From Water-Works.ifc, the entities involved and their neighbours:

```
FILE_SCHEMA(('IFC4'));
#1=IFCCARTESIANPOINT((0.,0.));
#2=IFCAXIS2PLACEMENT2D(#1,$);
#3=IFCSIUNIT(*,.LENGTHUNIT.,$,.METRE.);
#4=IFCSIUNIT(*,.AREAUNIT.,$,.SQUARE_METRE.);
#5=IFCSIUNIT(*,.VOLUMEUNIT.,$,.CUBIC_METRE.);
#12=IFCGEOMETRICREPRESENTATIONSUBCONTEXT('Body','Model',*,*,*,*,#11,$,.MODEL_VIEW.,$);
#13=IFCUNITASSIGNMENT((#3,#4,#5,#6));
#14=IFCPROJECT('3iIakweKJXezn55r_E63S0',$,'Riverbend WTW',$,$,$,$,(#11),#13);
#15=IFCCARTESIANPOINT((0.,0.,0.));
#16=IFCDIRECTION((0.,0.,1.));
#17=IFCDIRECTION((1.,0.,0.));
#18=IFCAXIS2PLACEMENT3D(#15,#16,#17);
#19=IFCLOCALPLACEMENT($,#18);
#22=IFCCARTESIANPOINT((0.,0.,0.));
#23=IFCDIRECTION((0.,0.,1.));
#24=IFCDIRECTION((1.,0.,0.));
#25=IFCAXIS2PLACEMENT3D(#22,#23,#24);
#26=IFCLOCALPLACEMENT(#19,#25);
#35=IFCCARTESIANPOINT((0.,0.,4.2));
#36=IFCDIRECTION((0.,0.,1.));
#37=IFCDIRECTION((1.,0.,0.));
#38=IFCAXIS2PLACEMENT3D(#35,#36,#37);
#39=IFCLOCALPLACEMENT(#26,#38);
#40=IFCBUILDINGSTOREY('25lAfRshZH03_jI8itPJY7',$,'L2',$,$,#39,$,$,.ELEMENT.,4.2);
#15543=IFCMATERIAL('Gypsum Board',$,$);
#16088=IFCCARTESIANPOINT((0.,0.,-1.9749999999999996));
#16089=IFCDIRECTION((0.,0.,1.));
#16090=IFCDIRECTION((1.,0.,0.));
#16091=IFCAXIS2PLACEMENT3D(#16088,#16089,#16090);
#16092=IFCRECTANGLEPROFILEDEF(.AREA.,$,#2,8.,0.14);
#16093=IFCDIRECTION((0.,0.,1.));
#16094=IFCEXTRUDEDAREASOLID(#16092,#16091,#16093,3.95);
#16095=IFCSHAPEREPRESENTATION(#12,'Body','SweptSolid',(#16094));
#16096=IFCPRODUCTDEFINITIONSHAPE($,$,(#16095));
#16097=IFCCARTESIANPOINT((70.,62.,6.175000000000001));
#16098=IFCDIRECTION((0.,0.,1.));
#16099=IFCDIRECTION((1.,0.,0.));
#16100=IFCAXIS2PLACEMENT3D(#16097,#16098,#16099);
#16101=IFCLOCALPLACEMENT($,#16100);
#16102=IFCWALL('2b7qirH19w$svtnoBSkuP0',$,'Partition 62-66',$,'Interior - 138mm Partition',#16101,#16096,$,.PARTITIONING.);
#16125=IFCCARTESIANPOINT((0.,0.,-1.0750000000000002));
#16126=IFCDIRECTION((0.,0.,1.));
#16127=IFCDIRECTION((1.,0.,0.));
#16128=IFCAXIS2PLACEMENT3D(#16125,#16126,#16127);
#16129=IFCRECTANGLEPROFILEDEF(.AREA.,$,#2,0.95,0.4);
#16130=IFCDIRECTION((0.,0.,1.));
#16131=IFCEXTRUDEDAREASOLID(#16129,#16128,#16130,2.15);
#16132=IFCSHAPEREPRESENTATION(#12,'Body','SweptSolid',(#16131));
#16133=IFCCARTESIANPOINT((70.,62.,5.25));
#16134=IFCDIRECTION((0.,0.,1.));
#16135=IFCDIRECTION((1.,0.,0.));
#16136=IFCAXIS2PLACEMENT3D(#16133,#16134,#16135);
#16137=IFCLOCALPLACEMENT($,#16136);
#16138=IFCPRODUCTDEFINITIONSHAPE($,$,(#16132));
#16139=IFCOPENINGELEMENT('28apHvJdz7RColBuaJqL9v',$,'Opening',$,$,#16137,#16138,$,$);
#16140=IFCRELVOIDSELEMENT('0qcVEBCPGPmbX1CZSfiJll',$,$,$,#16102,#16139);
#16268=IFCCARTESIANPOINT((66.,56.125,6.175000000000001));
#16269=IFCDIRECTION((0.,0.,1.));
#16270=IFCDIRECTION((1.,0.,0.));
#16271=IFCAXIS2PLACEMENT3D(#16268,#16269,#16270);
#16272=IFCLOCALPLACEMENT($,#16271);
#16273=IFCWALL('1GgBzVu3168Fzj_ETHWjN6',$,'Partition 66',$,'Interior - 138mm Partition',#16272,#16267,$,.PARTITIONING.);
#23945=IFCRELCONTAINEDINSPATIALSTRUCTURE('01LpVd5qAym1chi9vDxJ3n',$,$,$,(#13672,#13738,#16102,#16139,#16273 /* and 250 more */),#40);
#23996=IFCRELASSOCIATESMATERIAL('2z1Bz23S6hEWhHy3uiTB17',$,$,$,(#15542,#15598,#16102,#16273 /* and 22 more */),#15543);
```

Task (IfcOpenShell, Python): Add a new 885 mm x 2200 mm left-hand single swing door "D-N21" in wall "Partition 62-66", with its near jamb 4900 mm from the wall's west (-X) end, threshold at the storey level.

```python
import numpy as np
import ifcopenshell
import ifcopenshell.api.feature
import ifcopenshell.api.geometry
import ifcopenshell.api.root
import ifcopenshell.api.spatial
import ifcopenshell.geom
import ifcopenshell.util.element
import ifcopenshell.util.placement
import ifcopenshell.util.representation
import ifcopenshell.util.shape
import ifcopenshell.util.unit

model = ifcopenshell.open("Water-Works.ifc")
unit_scale = ifcopenshell.util.unit.calculate_unit_scale(model)
settings = ifcopenshell.geom.settings()


def volume(element):
    """Net volume in cubic metres, openings subtracted."""
    shape = ifcopenshell.geom.create_shape(settings, element)
    return ifcopenshell.util.shape.get_volume(shape.geometry)


wall = model.by_guid("2b7qirH19w$svtnoBSkuP0")
storey = ifcopenshell.util.element.get_container(wall, ifc_class="IfcBuildingStorey")
context = ifcopenshell.util.representation.get_context(model, "Model", "Body", "MODEL_VIEW")
before = volume(wall)

width, height, from_end, sill = 0.885, 2.2, 4.9, 0.0  # metres

# The wall runs along its own X axis, and the end named is its -X end.
wall_shape = ifcopenshell.geom.create_shape(settings, wall)
x, y, z = ifcopenshell.util.shape.get_vertices(wall_shape.geometry).T
start = x.min() + from_end
face, thickness = float(y.min()), float(y.max() - y.min())
wall_matrix = ifcopenshell.util.placement.get_local_placement(wall.ObjectPlacement)
level = ifcopenshell.util.placement.get_local_placement(storey.ObjectPlacement)[2, 3]


def in_wall(x, y):
    """Placement at x, y metres in the wall's axes, at sill height."""
    matrix = wall_matrix.copy()
    matrix[:, 3] = wall_matrix @ np.array([x / unit_scale, y / unit_scale, 0.0, 1.0])
    matrix[2, 3] = level + sill / unit_scale
    return matrix


# Opening: a box that overshoots both wall faces by 50 mm.
opening = ifcopenshell.api.root.create_entity(model, ifc_class="IfcOpeningElement", predefined_type="OPENING")
box = ifcopenshell.api.geometry.add_wall_representation(
    model, context=context, length=width, height=height, thickness=thickness + 0.1
)
ifcopenshell.api.geometry.assign_representation(model, product=opening, representation=box)
ifcopenshell.api.geometry.edit_object_placement(model, product=opening, matrix=in_wall(start, face - 0.05), is_si=False)
ifcopenshell.api.feature.add_feature(model, feature=opening, element=wall)

door = ifcopenshell.api.root.create_entity(model, ifc_class="IfcDoor", name="D-N21", predefined_type="DOOR")
door.OverallWidth, door.OverallHeight = width / unit_scale, height / unit_scale
door.OperationType = "SINGLE_SWING_LEFT"
body = ifcopenshell.api.geometry.add_door_representation(
    model,
    context=context,
    overall_width=door.OverallWidth,
    overall_height=door.OverallHeight,
    operation_type="SINGLE_SWING_LEFT",
    lining_properties={"LiningDepth": thickness / unit_scale, "ThresholdDepth": thickness / unit_scale},
)
ifcopenshell.api.geometry.assign_representation(model, product=door, representation=body)
ifcopenshell.api.spatial.assign_container(model, products=[door], relating_structure=storey)
ifcopenshell.api.feature.add_filling(model, opening=opening, element=door)

# The lining spans the wall, so the door starts at the wall face.
ifcopenshell.api.geometry.edit_object_placement(model, product=door, matrix=in_wall(start, face), is_si=False)

after = volume(wall)

print(f"wall volume {before:.3f} -> {after:.3f} m3")

model.write("Water-Works_rev.ifc")
```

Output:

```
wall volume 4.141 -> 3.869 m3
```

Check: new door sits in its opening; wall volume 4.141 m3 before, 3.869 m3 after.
